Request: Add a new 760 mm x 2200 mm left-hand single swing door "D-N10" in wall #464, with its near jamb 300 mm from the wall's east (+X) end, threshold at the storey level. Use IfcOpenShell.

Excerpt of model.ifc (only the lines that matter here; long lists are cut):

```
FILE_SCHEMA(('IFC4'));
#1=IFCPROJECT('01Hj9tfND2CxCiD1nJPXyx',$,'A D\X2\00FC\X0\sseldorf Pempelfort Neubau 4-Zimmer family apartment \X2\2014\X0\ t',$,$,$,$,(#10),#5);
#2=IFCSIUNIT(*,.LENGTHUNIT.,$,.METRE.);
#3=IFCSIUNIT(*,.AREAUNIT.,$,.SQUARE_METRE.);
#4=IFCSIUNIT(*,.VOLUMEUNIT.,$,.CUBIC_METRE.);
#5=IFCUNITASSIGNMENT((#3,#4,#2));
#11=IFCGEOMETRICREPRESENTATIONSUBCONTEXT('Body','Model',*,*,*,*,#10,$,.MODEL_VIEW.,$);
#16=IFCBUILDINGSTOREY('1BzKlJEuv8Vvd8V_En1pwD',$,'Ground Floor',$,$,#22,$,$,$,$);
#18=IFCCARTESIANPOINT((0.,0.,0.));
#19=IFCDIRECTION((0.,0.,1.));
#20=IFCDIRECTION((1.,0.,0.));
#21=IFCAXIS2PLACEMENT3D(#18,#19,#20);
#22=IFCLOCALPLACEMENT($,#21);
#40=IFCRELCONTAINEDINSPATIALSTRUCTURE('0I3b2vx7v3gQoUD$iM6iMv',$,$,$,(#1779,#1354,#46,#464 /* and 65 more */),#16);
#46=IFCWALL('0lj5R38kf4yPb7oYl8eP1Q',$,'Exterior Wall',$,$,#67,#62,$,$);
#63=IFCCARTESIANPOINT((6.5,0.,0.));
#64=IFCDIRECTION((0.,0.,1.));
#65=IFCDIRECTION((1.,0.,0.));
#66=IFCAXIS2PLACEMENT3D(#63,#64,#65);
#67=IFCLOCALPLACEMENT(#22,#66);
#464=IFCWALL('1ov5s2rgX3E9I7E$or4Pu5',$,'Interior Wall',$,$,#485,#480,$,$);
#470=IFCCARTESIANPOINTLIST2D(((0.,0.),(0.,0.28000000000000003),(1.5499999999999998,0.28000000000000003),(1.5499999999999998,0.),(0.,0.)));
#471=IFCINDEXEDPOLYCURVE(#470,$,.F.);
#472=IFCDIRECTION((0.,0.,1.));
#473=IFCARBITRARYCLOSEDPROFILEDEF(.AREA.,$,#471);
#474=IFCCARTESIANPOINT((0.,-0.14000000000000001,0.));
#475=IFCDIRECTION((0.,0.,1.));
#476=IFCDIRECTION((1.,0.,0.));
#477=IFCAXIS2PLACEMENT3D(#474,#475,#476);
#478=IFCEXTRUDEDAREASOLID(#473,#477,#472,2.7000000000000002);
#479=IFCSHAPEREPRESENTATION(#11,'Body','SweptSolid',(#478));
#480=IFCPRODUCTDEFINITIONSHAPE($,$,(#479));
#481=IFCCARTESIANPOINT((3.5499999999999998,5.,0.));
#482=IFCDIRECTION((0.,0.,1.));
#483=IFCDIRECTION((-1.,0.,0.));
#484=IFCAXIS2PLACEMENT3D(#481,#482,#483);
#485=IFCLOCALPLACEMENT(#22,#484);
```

```python
import numpy as np
import ifcopenshell
import ifcopenshell.api.feature
import ifcopenshell.api.geometry
import ifcopenshell.api.root
import ifcopenshell.api.spatial
import ifcopenshell.geom
import ifcopenshell.util.element
import ifcopenshell.util.placement
import ifcopenshell.util.representation
import ifcopenshell.util.shape
import ifcopenshell.util.unit

model = ifcopenshell.open("model.ifc")
unit_scale = ifcopenshell.util.unit.calculate_unit_scale(model)
settings = ifcopenshell.geom.settings()


def volume(element):
    """Net volume in cubic metres, openings subtracted."""
    shape = ifcopenshell.geom.create_shape(settings, element)
    return ifcopenshell.util.shape.get_volume(shape.geometry)


wall = model.by_guid("1ov5s2rgX3E9I7E$or4Pu5")
storey = ifcopenshell.util.element.get_container(wall, ifc_class="IfcBuildingStorey")
context = ifcopenshell.util.representation.get_context(model, "Model", "Body", "MODEL_VIEW")
before = volume(wall)

width, height, from_end, sill = 0.76, 2.2, 0.3, 0.0  # metres

# The wall runs along its own X axis, and the end named is its -X end.
wall_shape = ifcopenshell.geom.create_shape(settings, wall)
x, y, z = ifcopenshell.util.shape.get_vertices(wall_shape.geometry).T
start = x.min() + from_end
face, thickness = float(y.min()), float(y.max() - y.min())
wall_matrix = ifcopenshell.util.placement.get_local_placement(wall.ObjectPlacement)
level = ifcopenshell.util.placement.get_local_placement(storey.ObjectPlacement)[2, 3]


def in_wall(x, y):
    """Placement at x, y metres in the wall's axes, at sill height."""
    matrix = wall_matrix.copy()
    matrix[:, 3] = wall_matrix @ np.array([x / unit_scale, y / unit_scale, 0.0, 1.0])
    matrix[2, 3] = level + sill / unit_scale
    return matrix


# Opening: a box that overshoots both wall faces by 50 mm.
opening = ifcopenshell.api.root.create_entity(model, ifc_class="IfcOpeningElement", predefined_type="OPENING")
box = ifcopenshell.api.geometry.add_wall_representation(
    model, context=context, length=width, height=height, thickness=thickness + 0.1
)
ifcopenshell.api.geometry.assign_representation(model, product=opening, representation=box)
ifcopenshell.api.geometry.edit_object_placement(model, product=opening, matrix=in_wall(start, face - 0.05), is_si=False)
ifcopenshell.api.feature.add_feature(model, feature=opening, element=wall)

door = ifcopenshell.api.root.create_entity(model, ifc_class="IfcDoor", name="D-N10", predefined_type="DOOR")
door.OverallWidth, door.OverallHeight = width / unit_scale, height / unit_scale
door.OperationType = "SINGLE_SWING_LEFT"
body = ifcopenshell.api.geometry.add_door_representation(
    model,
    context=context,
    overall_width=door.OverallWidth,
    overall_height=door.OverallHeight,
    operation_type="SINGLE_SWING_LEFT",
    lining_properties={"LiningDepth": thickness / unit_scale, "ThresholdDepth": thickness / unit_scale},
)
ifcopenshell.api.geometry.assign_representation(model, product=door, representation=body)
ifcopenshell.api.spatial.assign_container(model, products=[door], relating_structure=storey)
ifcopenshell.api.feature.add_filling(model, opening=opening, element=door)

# The lining spans the wall, so the door starts at the wall face.
ifcopenshell.api.geometry.edit_object_placement(model, product=door, matrix=in_wall(start, face), is_si=False)

after = volume(wall)

print(f"wall volume {before:.3f} -> {after:.3f} m3")

model.write("model_rev.ifc")
```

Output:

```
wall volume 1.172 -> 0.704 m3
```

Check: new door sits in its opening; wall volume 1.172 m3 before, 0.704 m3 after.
